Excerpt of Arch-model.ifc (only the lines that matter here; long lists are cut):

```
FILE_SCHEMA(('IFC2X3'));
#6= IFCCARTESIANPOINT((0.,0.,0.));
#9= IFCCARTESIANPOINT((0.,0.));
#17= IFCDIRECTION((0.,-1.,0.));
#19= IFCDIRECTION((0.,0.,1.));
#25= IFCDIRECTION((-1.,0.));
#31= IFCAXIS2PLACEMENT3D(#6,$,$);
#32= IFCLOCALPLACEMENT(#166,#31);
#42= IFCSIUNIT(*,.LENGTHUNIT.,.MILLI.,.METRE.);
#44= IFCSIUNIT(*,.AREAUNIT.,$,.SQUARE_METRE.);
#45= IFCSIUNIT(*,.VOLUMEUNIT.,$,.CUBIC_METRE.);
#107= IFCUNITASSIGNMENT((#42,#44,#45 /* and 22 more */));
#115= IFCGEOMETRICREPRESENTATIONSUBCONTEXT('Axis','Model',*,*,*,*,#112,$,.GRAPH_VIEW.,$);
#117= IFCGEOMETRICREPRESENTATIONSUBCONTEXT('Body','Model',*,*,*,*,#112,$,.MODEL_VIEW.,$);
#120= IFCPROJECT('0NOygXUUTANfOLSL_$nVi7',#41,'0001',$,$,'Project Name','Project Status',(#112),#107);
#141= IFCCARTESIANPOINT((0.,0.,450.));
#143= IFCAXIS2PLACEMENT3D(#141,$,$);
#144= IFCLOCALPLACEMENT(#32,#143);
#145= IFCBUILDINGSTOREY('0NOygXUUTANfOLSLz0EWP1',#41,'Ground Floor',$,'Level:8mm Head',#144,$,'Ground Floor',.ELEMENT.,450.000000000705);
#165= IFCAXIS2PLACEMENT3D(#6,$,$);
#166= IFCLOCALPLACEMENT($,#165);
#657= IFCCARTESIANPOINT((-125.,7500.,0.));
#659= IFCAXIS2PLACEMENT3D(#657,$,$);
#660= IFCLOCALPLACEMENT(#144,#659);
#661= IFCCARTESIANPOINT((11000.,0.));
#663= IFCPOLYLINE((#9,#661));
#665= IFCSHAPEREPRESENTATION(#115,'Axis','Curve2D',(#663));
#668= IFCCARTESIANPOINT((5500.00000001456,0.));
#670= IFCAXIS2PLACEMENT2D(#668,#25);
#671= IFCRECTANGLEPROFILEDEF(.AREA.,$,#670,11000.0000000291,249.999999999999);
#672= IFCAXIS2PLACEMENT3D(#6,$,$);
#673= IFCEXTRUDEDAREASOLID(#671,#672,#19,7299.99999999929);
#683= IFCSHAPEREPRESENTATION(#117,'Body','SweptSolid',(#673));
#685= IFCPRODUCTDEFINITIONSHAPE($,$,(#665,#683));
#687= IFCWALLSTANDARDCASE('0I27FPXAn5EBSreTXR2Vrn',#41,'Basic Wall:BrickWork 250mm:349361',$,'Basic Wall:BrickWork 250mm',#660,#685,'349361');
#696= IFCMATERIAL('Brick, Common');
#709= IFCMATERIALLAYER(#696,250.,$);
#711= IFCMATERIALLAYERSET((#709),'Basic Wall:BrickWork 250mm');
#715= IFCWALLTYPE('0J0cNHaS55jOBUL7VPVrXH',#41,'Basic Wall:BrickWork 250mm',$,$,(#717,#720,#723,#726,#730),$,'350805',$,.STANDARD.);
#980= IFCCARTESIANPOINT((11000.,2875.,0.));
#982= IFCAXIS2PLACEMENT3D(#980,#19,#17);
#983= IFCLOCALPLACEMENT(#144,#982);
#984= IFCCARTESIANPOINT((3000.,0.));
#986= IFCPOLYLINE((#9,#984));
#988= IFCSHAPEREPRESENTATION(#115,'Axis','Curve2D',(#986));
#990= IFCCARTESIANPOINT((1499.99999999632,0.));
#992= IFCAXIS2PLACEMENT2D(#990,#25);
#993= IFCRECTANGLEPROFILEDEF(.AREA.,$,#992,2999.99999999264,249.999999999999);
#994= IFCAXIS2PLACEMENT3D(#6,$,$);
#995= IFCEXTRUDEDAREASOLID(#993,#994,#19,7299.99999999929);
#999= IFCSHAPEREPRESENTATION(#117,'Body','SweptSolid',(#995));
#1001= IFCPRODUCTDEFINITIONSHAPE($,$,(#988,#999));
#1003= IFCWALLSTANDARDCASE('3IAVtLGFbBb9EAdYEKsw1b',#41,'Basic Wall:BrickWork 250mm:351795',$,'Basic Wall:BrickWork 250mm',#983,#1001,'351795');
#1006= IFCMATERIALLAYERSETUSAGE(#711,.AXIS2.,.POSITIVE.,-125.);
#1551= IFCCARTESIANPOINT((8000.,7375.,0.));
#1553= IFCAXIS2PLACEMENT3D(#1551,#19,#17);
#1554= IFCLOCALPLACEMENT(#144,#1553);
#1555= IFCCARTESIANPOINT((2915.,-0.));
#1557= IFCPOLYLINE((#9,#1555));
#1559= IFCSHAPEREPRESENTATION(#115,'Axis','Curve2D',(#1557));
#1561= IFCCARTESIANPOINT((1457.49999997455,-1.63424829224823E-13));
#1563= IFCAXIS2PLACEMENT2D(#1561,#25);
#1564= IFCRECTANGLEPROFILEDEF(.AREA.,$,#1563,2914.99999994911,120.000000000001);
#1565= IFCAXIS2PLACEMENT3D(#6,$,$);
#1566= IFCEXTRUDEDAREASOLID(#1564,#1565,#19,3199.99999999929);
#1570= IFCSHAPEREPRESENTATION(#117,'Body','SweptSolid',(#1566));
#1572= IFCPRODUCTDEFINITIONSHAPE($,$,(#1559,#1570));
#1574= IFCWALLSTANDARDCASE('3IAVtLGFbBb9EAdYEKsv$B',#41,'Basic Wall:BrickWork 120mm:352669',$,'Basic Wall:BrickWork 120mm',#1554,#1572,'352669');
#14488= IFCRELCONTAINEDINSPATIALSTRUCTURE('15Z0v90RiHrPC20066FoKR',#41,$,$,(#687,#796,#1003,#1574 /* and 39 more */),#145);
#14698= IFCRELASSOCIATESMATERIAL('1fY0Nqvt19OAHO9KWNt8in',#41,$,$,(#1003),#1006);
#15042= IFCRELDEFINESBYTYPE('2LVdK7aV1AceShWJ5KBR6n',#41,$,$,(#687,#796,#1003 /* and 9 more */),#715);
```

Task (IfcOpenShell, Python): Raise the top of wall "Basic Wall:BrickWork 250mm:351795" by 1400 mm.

```python
import ifcopenshell
import ifcopenshell.geom
import ifcopenshell.util.representation
import ifcopenshell.util.shape
import ifcopenshell.util.unit

model = ifcopenshell.open("Arch-model.ifc")
unit_scale = ifcopenshell.util.unit.calculate_unit_scale(model)
settings = ifcopenshell.geom.settings()


def volume(element):
    """Net volume in cubic metres, openings subtracted."""
    shape = ifcopenshell.geom.create_shape(settings, element)
    return ifcopenshell.util.shape.get_volume(shape.geometry)


wall = model.by_guid("3IAVtLGFbBb9EAdYEKsw1b")
before = volume(wall)

body = ifcopenshell.util.representation.get_representation(wall, "Model", "Body")
solid = body.Items[0]
old_height = solid.Depth
solid.Depth += 1.4 / unit_scale
after = volume(wall)

print(f"height {old_height:g} -> {solid.Depth:g}, volume {before:.3f} -> {after:.3f} m3")

model.write("Arch-model_updated.ifc")
```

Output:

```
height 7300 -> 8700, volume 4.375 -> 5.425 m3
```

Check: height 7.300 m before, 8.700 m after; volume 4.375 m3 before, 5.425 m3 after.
